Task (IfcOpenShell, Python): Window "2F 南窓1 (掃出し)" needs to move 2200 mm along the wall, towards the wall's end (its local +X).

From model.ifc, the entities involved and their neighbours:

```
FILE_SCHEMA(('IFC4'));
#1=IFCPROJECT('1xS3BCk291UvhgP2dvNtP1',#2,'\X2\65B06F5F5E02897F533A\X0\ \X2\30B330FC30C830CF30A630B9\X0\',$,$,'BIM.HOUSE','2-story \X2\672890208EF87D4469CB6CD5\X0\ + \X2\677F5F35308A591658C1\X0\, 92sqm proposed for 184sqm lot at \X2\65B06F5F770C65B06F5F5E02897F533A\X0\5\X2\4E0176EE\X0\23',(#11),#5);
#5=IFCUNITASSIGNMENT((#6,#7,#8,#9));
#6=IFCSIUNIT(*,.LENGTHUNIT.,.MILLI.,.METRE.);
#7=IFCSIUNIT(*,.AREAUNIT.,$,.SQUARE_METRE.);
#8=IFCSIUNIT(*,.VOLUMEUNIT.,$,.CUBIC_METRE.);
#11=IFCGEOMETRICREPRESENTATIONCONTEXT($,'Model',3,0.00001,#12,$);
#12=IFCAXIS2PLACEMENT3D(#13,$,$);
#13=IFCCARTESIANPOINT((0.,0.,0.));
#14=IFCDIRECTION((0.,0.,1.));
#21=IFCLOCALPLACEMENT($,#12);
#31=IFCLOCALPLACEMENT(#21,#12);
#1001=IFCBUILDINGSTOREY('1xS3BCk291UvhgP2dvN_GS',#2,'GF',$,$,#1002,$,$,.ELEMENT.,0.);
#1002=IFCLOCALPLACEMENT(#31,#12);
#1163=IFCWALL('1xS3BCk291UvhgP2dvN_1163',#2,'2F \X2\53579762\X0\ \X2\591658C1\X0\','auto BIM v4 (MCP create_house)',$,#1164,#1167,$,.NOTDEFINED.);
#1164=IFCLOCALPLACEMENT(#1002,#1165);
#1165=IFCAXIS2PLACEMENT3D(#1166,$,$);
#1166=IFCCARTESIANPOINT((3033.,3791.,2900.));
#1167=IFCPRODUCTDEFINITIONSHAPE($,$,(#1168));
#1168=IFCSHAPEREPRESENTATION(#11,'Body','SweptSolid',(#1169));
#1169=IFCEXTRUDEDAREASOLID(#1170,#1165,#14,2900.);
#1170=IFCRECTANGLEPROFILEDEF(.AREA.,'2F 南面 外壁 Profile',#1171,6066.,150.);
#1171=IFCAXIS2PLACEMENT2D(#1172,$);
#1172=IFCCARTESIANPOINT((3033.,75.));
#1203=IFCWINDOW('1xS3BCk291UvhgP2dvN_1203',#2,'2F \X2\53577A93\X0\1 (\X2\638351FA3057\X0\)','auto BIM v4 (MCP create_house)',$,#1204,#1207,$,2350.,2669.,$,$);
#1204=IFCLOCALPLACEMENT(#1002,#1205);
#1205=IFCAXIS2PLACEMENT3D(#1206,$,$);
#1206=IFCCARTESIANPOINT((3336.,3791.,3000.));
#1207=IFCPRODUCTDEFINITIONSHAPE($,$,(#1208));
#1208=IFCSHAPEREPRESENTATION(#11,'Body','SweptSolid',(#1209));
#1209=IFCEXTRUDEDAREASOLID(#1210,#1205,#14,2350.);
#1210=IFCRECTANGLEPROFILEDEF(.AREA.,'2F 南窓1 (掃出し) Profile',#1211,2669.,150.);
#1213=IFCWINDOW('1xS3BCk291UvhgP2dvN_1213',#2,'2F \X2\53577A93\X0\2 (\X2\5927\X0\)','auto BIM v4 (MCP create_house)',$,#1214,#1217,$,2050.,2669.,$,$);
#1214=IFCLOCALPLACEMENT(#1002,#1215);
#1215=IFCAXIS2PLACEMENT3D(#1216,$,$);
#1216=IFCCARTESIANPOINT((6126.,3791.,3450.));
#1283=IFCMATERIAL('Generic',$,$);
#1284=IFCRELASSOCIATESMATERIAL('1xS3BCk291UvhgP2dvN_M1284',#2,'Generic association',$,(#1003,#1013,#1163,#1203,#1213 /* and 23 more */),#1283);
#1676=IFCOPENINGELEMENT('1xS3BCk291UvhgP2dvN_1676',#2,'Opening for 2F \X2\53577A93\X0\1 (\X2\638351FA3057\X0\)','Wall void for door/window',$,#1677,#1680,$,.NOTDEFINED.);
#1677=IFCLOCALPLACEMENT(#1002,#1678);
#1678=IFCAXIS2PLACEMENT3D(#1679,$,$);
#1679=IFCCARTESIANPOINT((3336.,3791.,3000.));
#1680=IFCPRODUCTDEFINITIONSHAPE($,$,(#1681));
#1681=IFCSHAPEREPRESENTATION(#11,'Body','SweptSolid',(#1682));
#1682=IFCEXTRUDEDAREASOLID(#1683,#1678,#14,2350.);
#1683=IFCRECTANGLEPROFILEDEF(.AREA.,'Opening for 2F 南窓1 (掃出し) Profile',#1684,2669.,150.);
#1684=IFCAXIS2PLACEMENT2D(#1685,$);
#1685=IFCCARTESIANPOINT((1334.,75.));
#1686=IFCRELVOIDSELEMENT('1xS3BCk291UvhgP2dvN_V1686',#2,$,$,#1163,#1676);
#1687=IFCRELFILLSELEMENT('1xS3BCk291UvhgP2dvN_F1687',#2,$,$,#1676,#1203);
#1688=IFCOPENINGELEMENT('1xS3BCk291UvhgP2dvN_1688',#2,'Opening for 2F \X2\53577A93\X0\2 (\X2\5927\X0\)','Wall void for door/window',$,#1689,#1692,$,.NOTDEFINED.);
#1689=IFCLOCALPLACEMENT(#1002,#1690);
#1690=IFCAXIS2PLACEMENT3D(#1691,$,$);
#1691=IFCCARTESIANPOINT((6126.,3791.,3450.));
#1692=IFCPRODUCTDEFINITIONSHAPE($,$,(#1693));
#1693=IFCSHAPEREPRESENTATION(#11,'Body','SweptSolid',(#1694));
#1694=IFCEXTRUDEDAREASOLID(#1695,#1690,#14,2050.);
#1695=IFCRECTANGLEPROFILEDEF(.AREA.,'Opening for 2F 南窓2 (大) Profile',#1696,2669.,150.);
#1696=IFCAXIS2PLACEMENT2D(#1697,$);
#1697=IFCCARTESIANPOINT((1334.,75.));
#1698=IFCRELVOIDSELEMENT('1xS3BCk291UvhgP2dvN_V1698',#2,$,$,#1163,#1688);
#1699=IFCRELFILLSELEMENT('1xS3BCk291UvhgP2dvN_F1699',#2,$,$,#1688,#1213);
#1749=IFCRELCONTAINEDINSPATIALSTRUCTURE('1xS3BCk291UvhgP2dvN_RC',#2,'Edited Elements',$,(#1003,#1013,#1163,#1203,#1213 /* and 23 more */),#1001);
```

```python
import ifcopenshell
import ifcopenshell.api.geometry
import ifcopenshell.util.placement

model = ifcopenshell.open("model.ifc")

window = model.by_id(1203)
opening = window.FillsVoids[0].RelatingOpeningElement
wall = opening.VoidsElements[0].RelatingBuildingElement

wall_matrix = ifcopenshell.util.placement.get_local_placement(wall.ObjectPlacement)
shift = wall_matrix[:3, 0] * 2200.0
before = ifcopenshell.util.placement.get_local_placement(window.ObjectPlacement)[:3, 3].copy()

# The window is not placed relative to its opening, so move both.
for product in (opening, window):
    matrix = ifcopenshell.util.placement.get_local_placement(product.ObjectPlacement)
    matrix[:3, 3] += shift
    ifcopenshell.api.geometry.edit_object_placement(model, product=product, matrix=matrix, is_si=False)

after = ifcopenshell.util.placement.get_local_placement(window.ObjectPlacement)[:3, 3]
print("window moved by", (after - before).round(3) + 0.0)

model.write("model_v2.ifc")
```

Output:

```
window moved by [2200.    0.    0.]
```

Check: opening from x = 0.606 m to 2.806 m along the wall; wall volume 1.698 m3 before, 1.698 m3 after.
